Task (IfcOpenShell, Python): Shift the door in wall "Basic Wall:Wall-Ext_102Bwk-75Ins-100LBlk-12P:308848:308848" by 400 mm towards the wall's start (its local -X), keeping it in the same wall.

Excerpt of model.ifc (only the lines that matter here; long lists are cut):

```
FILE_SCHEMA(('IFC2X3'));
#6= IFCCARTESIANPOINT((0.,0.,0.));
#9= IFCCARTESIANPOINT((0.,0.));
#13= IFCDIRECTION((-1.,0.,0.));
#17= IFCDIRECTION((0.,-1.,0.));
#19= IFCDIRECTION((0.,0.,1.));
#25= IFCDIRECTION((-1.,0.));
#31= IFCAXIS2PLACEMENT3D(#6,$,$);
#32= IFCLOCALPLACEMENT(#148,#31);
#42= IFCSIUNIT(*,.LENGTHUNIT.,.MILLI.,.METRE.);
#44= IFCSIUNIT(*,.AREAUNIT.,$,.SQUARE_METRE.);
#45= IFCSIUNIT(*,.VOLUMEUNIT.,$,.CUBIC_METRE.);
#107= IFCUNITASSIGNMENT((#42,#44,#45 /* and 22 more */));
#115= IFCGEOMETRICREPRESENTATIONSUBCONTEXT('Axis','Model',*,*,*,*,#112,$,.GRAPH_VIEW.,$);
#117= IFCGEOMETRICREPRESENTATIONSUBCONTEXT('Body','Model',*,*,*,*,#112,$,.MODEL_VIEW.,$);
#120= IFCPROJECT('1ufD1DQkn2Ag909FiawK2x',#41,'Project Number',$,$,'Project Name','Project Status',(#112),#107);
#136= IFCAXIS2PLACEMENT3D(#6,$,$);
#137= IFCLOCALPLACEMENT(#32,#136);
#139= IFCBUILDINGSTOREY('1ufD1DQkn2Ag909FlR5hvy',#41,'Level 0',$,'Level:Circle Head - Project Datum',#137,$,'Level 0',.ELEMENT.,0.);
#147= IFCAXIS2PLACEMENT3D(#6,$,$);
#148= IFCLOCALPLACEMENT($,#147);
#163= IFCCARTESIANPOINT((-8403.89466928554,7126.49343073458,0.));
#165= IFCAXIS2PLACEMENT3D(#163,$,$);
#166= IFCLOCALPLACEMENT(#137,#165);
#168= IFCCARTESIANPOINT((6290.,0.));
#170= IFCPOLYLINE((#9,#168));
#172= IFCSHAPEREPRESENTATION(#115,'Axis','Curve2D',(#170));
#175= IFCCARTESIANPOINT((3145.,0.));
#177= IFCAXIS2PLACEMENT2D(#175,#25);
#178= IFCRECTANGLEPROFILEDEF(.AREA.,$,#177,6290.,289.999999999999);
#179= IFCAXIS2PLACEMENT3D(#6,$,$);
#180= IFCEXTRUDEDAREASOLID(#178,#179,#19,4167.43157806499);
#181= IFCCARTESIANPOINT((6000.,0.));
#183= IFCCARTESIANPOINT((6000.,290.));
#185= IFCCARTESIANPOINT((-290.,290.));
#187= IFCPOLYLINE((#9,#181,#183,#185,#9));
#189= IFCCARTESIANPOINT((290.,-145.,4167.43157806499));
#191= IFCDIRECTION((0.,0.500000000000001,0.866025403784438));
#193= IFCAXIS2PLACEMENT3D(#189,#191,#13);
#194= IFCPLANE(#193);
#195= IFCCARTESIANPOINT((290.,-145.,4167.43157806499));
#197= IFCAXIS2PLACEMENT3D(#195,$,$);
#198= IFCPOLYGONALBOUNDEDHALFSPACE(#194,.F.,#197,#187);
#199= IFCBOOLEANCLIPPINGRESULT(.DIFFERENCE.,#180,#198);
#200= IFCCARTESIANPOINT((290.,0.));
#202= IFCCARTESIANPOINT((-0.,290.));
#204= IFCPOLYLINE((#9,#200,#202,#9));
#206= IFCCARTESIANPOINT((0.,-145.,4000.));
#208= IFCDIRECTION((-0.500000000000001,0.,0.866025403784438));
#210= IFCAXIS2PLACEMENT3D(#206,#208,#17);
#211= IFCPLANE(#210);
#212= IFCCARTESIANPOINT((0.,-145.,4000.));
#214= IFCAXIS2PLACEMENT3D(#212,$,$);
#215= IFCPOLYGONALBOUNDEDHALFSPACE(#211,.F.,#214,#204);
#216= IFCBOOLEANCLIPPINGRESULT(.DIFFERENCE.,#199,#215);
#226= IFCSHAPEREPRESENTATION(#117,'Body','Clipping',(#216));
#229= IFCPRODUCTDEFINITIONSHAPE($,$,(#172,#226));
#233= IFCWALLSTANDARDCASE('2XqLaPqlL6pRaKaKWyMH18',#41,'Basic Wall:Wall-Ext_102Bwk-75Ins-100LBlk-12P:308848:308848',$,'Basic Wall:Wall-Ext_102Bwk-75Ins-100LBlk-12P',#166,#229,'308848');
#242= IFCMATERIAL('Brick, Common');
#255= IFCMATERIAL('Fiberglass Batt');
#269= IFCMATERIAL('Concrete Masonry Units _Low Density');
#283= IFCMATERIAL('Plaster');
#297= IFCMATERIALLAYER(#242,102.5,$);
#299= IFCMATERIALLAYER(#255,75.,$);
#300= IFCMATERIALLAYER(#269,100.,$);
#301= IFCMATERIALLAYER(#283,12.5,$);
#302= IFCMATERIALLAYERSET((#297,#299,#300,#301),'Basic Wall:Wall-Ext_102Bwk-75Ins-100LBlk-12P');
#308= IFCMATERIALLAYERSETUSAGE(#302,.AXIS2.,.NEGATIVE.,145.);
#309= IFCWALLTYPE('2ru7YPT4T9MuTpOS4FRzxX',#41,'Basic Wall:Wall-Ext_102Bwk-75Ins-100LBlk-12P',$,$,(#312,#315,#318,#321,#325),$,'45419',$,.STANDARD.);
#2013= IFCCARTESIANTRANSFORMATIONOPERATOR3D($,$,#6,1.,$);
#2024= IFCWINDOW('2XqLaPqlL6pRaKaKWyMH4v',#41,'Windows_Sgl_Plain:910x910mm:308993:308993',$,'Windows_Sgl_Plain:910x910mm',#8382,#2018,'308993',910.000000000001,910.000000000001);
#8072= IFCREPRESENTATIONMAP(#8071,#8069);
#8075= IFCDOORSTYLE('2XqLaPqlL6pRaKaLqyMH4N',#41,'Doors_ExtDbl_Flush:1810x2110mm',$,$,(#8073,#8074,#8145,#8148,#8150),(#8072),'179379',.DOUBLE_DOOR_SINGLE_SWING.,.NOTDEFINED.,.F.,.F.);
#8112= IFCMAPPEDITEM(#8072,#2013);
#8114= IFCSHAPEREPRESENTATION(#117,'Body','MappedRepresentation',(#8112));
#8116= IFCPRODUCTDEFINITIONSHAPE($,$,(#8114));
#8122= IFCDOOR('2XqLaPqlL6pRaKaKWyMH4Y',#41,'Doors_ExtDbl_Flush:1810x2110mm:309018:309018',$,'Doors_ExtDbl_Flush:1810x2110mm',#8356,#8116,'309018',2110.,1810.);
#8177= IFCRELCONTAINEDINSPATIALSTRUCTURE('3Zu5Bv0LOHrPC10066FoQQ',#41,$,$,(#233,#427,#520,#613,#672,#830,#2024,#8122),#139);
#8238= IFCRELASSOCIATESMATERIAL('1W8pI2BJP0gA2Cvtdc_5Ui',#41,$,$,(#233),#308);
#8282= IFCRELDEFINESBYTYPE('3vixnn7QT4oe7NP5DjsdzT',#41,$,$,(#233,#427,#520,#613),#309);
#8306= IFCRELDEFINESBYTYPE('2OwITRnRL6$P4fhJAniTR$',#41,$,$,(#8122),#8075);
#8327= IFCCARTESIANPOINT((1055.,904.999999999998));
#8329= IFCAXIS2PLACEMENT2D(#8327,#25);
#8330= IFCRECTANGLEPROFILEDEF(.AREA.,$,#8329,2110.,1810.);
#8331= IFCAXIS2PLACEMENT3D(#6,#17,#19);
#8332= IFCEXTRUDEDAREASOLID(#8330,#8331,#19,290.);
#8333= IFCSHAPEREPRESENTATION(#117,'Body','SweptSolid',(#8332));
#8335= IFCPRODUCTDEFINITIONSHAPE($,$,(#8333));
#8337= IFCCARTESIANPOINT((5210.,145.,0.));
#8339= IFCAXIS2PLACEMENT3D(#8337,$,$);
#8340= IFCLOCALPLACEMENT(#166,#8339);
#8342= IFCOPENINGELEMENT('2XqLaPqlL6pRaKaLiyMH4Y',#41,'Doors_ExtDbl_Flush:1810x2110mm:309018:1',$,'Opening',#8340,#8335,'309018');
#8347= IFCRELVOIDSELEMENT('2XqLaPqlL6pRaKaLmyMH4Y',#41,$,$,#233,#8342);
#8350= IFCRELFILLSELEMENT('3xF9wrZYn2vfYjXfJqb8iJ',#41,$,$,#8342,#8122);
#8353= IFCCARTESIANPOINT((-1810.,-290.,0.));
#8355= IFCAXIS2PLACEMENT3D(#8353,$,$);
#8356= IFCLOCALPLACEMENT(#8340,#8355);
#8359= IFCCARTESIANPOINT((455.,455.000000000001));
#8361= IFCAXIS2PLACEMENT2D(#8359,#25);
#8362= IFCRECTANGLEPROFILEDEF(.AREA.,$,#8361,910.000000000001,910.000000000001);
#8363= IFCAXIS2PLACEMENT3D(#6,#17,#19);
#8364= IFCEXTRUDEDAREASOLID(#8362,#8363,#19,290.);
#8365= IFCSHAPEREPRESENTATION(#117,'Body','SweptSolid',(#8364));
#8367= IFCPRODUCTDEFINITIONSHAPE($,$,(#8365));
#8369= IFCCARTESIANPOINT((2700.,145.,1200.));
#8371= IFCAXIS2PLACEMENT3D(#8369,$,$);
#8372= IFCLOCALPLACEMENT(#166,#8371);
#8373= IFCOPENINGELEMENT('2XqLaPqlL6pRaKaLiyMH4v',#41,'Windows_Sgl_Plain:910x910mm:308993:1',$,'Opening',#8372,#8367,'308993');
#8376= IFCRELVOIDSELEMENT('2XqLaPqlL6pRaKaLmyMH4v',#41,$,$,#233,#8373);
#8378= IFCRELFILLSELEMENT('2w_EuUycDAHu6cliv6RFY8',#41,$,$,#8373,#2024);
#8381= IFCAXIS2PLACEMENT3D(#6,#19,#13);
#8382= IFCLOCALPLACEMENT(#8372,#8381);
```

```python
import ifcopenshell
import ifcopenshell.api.geometry
import ifcopenshell.util.placement
import ifcopenshell.util.unit

model = ifcopenshell.open("model.ifc")
unit_scale = ifcopenshell.util.unit.calculate_unit_scale(model)

door = model.by_guid("2XqLaPqlL6pRaKaKWyMH4Y")
opening = door.FillsVoids[0].RelatingOpeningElement
wall = opening.VoidsElements[0].RelatingBuildingElement

wall_matrix = ifcopenshell.util.placement.get_local_placement(wall.ObjectPlacement)
shift = wall_matrix[:3, 0] * -0.4 / unit_scale
before = ifcopenshell.util.placement.get_local_placement(door.ObjectPlacement)[:3, 3].copy()

# The door is placed relative to its opening, so it follows when the opening moves.
matrix = ifcopenshell.util.placement.get_local_placement(opening.ObjectPlacement)
matrix[:3, 3] += shift
ifcopenshell.api.geometry.edit_object_placement(
    model, product=opening, matrix=matrix, is_si=False, should_transform_children=True
)

after = ifcopenshell.util.placement.get_local_placement(door.ObjectPlacement)[:3, 3]
print("door moved by", (after - before).round(3) + 0.0)

model.write("model_rev.ifc")
```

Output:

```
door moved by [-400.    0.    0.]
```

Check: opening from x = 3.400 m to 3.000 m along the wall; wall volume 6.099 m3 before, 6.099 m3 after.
